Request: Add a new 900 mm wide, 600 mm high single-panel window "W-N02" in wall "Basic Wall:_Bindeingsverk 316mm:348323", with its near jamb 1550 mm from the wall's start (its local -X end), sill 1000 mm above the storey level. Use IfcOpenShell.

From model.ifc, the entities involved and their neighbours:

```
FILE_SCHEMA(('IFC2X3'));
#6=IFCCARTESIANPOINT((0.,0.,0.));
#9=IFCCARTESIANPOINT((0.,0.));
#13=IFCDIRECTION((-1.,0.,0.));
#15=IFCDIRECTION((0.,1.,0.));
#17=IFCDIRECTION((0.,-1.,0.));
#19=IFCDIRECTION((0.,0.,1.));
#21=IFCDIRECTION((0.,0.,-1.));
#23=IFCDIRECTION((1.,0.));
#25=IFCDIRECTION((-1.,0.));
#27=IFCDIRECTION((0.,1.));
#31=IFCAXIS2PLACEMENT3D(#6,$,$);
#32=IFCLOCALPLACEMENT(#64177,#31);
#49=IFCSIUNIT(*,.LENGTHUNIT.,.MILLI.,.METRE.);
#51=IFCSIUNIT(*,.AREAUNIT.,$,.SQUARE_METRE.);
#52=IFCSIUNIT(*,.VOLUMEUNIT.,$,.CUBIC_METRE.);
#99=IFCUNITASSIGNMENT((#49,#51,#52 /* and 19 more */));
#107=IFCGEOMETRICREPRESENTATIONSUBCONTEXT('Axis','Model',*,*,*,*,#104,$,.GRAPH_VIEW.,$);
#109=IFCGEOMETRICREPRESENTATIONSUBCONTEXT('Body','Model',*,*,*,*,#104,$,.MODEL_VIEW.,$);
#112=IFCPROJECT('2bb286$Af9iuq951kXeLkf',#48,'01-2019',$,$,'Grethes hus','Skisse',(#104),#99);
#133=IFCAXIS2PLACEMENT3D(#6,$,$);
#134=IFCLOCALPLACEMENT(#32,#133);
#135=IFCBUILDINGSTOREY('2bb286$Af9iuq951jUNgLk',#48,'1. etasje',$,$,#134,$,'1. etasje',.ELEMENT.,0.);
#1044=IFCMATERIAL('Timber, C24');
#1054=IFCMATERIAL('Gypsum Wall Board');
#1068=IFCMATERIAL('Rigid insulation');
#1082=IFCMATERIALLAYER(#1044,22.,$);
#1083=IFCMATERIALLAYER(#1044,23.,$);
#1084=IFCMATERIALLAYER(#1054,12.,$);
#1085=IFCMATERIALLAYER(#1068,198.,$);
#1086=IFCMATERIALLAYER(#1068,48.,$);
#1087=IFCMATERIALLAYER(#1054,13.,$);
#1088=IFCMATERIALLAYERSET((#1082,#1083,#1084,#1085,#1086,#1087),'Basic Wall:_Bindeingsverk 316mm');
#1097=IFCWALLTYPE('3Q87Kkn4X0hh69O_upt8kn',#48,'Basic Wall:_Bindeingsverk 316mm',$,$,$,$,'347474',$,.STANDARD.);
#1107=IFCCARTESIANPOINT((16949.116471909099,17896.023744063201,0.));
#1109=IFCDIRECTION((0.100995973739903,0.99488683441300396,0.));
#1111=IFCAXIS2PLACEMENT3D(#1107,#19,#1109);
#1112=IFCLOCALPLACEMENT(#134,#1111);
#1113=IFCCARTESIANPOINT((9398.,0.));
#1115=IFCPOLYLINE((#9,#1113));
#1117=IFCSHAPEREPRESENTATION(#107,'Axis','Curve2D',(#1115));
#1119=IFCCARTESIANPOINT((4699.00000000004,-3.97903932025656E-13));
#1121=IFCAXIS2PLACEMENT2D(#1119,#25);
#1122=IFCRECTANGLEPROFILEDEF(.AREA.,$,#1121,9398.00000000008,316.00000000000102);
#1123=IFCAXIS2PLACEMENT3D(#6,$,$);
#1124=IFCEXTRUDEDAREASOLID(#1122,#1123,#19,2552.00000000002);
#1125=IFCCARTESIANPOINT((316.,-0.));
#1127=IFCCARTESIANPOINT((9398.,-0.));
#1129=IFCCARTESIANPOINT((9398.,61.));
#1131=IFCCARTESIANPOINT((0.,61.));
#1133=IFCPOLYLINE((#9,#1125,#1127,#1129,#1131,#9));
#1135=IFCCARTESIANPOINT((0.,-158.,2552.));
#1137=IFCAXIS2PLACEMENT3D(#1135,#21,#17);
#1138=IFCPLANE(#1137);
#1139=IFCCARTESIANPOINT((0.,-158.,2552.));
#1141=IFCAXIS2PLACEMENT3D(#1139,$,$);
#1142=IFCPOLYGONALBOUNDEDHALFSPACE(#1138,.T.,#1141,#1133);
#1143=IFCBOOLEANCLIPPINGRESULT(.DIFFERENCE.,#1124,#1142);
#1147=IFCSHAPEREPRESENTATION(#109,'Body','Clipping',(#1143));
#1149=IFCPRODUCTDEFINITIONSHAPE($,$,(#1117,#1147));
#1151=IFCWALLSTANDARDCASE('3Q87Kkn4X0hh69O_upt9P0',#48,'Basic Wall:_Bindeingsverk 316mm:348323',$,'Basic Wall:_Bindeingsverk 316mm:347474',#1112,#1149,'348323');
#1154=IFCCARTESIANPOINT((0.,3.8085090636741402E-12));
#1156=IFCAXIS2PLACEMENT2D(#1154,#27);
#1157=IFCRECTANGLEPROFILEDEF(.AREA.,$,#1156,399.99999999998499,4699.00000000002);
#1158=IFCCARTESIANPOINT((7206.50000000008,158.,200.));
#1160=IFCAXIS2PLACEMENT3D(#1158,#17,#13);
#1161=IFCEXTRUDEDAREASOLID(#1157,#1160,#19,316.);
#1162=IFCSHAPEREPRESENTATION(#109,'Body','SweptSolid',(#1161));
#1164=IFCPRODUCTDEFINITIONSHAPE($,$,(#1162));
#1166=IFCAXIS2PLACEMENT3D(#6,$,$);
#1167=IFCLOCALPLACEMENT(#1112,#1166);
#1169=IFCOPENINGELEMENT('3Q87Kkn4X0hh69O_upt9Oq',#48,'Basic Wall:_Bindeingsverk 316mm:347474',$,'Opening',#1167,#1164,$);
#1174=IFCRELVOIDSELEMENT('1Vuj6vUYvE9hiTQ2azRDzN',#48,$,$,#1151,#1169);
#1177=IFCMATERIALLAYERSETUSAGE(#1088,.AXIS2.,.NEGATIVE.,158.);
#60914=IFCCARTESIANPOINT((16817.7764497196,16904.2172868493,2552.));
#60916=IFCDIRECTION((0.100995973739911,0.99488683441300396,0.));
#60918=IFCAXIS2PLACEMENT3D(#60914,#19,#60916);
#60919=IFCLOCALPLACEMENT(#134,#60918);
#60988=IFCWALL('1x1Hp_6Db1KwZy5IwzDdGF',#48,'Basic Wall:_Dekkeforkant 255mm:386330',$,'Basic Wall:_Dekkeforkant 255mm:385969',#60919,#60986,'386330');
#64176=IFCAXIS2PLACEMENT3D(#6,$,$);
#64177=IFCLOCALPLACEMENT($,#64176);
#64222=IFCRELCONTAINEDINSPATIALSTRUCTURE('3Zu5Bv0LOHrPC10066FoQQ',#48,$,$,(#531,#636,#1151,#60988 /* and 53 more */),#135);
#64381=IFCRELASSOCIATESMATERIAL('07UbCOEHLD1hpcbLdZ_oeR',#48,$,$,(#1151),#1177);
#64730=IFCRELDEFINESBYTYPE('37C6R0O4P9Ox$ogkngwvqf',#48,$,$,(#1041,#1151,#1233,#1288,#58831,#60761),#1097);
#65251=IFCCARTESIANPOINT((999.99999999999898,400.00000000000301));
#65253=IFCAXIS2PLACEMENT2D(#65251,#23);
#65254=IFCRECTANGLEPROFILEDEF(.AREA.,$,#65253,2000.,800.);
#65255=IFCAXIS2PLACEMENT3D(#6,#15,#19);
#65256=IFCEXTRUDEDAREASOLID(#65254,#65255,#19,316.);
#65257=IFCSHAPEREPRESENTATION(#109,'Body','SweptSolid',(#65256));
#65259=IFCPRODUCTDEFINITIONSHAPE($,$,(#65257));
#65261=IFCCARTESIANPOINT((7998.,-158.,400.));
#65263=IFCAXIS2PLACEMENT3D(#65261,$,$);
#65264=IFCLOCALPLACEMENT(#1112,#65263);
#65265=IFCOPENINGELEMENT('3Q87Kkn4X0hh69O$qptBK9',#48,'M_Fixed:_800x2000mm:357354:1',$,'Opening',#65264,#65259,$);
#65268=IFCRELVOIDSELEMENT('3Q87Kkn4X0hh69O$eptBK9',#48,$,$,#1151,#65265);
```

```python
import numpy as np
import ifcopenshell
import ifcopenshell.api.feature
import ifcopenshell.api.geometry
import ifcopenshell.api.root
import ifcopenshell.api.spatial
import ifcopenshell.api.type
import ifcopenshell.geom
import ifcopenshell.util.element
import ifcopenshell.util.placement
import ifcopenshell.util.representation
import ifcopenshell.util.shape
import ifcopenshell.util.unit

model = ifcopenshell.open("model.ifc")
unit_scale = ifcopenshell.util.unit.calculate_unit_scale(model)
settings = ifcopenshell.geom.settings()


def volume(element):
    """Net volume in cubic metres, openings subtracted."""
    shape = ifcopenshell.geom.create_shape(settings, element)
    return ifcopenshell.util.shape.get_volume(shape.geometry)


wall = model.by_id(1151)
storey = ifcopenshell.util.element.get_container(wall, ifc_class="IfcBuildingStorey")
context = ifcopenshell.util.representation.get_context(model, "Model", "Body", "MODEL_VIEW")
before = volume(wall)

width, height, from_end, sill = 0.9, 0.6, 1.55, 1  # metres

# The wall runs along its own X axis, and the end named is its -X end.
wall_shape = ifcopenshell.geom.create_shape(settings, wall)
x, y, z = ifcopenshell.util.shape.get_vertices(wall_shape.geometry).T
start = x.min() + from_end
face, thickness = float(y.min()), float(y.max() - y.min())
wall_matrix = ifcopenshell.util.placement.get_local_placement(wall.ObjectPlacement)
level = ifcopenshell.util.placement.get_local_placement(storey.ObjectPlacement)[2, 3]


def in_wall(x, y):
    """Placement at x, y metres in the wall's axes, at sill height."""
    matrix = wall_matrix.copy()
    matrix[:, 3] = wall_matrix @ np.array([x / unit_scale, y / unit_scale, 0.0, 1.0])
    matrix[2, 3] = level + sill / unit_scale
    return matrix


# Opening: a box that overshoots both wall faces by 50 mm.
opening = ifcopenshell.api.root.create_entity(model, ifc_class="IfcOpeningElement")
box = ifcopenshell.api.geometry.add_wall_representation(
    model, context=context, length=width, height=height, thickness=thickness + 0.1
)
ifcopenshell.api.geometry.assign_representation(model, product=opening, representation=box)
ifcopenshell.api.geometry.edit_object_placement(model, product=opening, matrix=in_wall(start, face - 0.05), is_si=False)
ifcopenshell.api.feature.add_feature(model, feature=opening, element=wall)

window = ifcopenshell.api.root.create_entity(model, ifc_class="IfcWindow", name="W-N02")
window.OverallWidth, window.OverallHeight = width / unit_scale, height / unit_scale
body = ifcopenshell.api.geometry.add_window_representation(
    model,
    context=context,
    overall_width=window.OverallWidth,
    overall_height=window.OverallHeight,
    partition_type="SINGLE_PANEL",
)
ifcopenshell.api.geometry.assign_representation(model, product=window, representation=body)
ifcopenshell.api.spatial.assign_container(model, products=[window], relating_structure=storey)
fills = ifcopenshell.api.feature.add_filling(model, opening=opening, element=window)
fills.OwnerHistory = window.OwnerHistory  # required in IFC2X3

# IFC2X3 keeps the operation on the window style.
style = ifcopenshell.api.root.create_entity(model, ifc_class="IfcWindowStyle", name="W-N02")
style.OperationType, style.ConstructionType = "SINGLE_PANEL", "NOTDEFINED"
style.ParameterTakesPrecedence = style.Sizeable = False
ifcopenshell.api.type.assign_type(model, related_objects=[window], relating_type=style)

# Centre the window in the wall's thickness.
ifcopenshell.api.geometry.edit_object_placement(model, product=window, matrix=in_wall(start, face), is_si=False)
window_shape = ifcopenshell.geom.create_shape(settings, window)
depth = ifcopenshell.util.shape.get_vertices(window_shape.geometry)[:, 1]
offset = face + thickness / 2 - (depth.min() + depth.max()) / 2
ifcopenshell.api.geometry.edit_object_placement(model, product=window, matrix=in_wall(start, offset), is_si=False)

after = volume(wall)

print(f"wall volume {before:.3f} -> {after:.3f} m3")

model.write("model_v2.ifc")
```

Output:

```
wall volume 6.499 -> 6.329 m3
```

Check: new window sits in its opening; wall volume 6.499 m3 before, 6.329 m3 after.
